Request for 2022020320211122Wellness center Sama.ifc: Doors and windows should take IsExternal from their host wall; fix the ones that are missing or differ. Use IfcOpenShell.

First a look at what the model holds.

```python
import ifcopenshell
import ifcopenshell.util.element

model = ifcopenshell.open("2022020320211122Wellness center Sama.ifc")
print(model.schema)
seen = {}
for e in model.by_type("IfcDoor") + model.by_type("IfcWindow"):
    if not e.FillsVoids:
        continue
    host = e.FillsVoids[0].RelatingOpeningElement.VoidsElements[0].RelatingBuildingElement
    own = ifcopenshell.util.element.get_pset(e, f"Pset_{e.is_a()[3:].removesuffix('StandardCase')}Common", "IsExternal")
    wall = ifcopenshell.util.element.get_pset(host, "Pset_WallCommon", "IsExternal")
    seen[e.is_a(), own, wall] = seen.get((e.is_a(), own, wall), 0) + 1
for (cls, own, wall), count in sorted(seen.items(), key=str):
    print(count, cls, "IsExternal:", own, "| host wall:", wall)
```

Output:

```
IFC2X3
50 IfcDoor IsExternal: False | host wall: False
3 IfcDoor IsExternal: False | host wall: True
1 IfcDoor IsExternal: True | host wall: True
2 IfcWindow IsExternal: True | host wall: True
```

```python
import ifcopenshell
import ifcopenshell.api.pset
import ifcopenshell.util.element

model = ifcopenshell.open("2022020320211122Wellness center Sama.ifc")

count = 0
for ifc_class, pset_name in (("IfcDoor", "Pset_DoorCommon"), ("IfcWindow", "Pset_WindowCommon")):
    for e in model.by_type(ifc_class):
        if not e.FillsVoids:
            continue
        host = e.FillsVoids[0].RelatingOpeningElement.VoidsElements[0].RelatingBuildingElement
        external = ifcopenshell.util.element.get_pset(host, "Pset_WallCommon", "IsExternal")
        if external is None or ifcopenshell.util.element.get_pset(e, pset_name, "IsExternal") == external:
            continue
        pset = ifcopenshell.api.pset.add_pset(model, product=e, name=pset_name)
        ifcopenshell.api.pset.edit_pset(model, pset=pset, properties={"IsExternal": external})
        count += 1

print(count, "updated")

model.write("2022020320211122Wellness center Sama_v2.ifc")
```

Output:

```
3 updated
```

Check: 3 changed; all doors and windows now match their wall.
